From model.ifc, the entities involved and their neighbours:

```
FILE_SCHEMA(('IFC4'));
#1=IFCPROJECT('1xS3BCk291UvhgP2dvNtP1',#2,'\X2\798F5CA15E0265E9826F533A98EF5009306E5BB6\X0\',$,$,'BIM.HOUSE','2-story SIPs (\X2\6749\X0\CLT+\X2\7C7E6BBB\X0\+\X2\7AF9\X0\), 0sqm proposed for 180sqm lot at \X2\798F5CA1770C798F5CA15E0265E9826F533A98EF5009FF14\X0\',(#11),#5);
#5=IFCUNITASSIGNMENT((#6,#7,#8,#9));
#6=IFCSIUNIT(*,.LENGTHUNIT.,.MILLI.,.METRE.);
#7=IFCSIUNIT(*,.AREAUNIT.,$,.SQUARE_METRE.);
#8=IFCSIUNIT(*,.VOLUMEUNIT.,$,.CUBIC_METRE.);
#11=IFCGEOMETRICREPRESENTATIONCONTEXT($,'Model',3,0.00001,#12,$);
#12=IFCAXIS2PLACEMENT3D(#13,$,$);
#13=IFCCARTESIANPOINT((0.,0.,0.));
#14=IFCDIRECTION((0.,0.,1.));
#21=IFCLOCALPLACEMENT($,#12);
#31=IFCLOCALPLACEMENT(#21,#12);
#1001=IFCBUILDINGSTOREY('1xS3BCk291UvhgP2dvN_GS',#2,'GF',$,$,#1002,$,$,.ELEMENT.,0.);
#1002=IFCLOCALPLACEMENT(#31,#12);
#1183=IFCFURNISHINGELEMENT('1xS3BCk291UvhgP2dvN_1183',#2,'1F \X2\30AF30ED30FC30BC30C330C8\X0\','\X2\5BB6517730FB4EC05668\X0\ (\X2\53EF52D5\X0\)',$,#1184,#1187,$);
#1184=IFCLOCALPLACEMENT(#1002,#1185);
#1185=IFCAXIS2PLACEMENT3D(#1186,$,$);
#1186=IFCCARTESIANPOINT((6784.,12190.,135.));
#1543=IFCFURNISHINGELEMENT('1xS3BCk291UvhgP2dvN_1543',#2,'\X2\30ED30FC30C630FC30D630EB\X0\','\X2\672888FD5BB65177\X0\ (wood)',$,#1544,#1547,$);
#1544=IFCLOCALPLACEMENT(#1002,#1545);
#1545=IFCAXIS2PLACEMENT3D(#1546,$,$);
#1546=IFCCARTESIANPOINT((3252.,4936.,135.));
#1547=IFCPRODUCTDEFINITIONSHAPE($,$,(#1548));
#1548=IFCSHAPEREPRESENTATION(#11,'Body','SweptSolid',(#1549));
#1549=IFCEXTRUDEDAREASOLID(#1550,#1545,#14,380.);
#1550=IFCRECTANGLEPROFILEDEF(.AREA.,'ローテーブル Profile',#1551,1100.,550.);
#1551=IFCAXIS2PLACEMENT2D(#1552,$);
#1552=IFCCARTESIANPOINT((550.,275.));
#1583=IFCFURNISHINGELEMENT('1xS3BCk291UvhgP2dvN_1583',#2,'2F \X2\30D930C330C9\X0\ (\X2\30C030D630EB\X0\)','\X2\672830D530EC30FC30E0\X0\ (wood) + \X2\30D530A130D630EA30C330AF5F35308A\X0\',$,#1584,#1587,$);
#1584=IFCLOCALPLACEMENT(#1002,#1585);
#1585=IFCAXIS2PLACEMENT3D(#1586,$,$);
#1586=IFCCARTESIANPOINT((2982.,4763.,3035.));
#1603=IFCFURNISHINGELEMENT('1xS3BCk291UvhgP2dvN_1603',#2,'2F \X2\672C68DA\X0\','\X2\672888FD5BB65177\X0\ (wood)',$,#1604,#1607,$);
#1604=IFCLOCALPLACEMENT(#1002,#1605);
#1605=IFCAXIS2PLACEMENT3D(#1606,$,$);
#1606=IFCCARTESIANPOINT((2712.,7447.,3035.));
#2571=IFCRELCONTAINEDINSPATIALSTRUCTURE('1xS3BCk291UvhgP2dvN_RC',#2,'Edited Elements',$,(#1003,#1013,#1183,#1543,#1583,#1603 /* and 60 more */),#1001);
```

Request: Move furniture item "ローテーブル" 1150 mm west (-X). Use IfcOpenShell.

```python
import ifcopenshell
import ifcopenshell.api.geometry
import ifcopenshell.util.placement
import ifcopenshell.util.unit

model = ifcopenshell.open("model.ifc")
unit_scale = ifcopenshell.util.unit.calculate_unit_scale(model)

item = model.by_guid("1xS3BCk291UvhgP2dvN_1543")
matrix = ifcopenshell.util.placement.get_local_placement(item.ObjectPlacement)
matrix[0, 3] -= 1.15 / unit_scale
ifcopenshell.api.geometry.edit_object_placement(model, product=item, matrix=matrix, is_si=False)

print(ifcopenshell.util.placement.get_local_placement(item.ObjectPlacement).round(3) + 0.0)

model.write("model_updated.ifc")
```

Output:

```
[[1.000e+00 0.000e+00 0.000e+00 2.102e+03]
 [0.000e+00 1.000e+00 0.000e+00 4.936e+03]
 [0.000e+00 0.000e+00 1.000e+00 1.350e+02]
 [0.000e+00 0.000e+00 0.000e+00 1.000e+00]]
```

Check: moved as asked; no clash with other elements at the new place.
